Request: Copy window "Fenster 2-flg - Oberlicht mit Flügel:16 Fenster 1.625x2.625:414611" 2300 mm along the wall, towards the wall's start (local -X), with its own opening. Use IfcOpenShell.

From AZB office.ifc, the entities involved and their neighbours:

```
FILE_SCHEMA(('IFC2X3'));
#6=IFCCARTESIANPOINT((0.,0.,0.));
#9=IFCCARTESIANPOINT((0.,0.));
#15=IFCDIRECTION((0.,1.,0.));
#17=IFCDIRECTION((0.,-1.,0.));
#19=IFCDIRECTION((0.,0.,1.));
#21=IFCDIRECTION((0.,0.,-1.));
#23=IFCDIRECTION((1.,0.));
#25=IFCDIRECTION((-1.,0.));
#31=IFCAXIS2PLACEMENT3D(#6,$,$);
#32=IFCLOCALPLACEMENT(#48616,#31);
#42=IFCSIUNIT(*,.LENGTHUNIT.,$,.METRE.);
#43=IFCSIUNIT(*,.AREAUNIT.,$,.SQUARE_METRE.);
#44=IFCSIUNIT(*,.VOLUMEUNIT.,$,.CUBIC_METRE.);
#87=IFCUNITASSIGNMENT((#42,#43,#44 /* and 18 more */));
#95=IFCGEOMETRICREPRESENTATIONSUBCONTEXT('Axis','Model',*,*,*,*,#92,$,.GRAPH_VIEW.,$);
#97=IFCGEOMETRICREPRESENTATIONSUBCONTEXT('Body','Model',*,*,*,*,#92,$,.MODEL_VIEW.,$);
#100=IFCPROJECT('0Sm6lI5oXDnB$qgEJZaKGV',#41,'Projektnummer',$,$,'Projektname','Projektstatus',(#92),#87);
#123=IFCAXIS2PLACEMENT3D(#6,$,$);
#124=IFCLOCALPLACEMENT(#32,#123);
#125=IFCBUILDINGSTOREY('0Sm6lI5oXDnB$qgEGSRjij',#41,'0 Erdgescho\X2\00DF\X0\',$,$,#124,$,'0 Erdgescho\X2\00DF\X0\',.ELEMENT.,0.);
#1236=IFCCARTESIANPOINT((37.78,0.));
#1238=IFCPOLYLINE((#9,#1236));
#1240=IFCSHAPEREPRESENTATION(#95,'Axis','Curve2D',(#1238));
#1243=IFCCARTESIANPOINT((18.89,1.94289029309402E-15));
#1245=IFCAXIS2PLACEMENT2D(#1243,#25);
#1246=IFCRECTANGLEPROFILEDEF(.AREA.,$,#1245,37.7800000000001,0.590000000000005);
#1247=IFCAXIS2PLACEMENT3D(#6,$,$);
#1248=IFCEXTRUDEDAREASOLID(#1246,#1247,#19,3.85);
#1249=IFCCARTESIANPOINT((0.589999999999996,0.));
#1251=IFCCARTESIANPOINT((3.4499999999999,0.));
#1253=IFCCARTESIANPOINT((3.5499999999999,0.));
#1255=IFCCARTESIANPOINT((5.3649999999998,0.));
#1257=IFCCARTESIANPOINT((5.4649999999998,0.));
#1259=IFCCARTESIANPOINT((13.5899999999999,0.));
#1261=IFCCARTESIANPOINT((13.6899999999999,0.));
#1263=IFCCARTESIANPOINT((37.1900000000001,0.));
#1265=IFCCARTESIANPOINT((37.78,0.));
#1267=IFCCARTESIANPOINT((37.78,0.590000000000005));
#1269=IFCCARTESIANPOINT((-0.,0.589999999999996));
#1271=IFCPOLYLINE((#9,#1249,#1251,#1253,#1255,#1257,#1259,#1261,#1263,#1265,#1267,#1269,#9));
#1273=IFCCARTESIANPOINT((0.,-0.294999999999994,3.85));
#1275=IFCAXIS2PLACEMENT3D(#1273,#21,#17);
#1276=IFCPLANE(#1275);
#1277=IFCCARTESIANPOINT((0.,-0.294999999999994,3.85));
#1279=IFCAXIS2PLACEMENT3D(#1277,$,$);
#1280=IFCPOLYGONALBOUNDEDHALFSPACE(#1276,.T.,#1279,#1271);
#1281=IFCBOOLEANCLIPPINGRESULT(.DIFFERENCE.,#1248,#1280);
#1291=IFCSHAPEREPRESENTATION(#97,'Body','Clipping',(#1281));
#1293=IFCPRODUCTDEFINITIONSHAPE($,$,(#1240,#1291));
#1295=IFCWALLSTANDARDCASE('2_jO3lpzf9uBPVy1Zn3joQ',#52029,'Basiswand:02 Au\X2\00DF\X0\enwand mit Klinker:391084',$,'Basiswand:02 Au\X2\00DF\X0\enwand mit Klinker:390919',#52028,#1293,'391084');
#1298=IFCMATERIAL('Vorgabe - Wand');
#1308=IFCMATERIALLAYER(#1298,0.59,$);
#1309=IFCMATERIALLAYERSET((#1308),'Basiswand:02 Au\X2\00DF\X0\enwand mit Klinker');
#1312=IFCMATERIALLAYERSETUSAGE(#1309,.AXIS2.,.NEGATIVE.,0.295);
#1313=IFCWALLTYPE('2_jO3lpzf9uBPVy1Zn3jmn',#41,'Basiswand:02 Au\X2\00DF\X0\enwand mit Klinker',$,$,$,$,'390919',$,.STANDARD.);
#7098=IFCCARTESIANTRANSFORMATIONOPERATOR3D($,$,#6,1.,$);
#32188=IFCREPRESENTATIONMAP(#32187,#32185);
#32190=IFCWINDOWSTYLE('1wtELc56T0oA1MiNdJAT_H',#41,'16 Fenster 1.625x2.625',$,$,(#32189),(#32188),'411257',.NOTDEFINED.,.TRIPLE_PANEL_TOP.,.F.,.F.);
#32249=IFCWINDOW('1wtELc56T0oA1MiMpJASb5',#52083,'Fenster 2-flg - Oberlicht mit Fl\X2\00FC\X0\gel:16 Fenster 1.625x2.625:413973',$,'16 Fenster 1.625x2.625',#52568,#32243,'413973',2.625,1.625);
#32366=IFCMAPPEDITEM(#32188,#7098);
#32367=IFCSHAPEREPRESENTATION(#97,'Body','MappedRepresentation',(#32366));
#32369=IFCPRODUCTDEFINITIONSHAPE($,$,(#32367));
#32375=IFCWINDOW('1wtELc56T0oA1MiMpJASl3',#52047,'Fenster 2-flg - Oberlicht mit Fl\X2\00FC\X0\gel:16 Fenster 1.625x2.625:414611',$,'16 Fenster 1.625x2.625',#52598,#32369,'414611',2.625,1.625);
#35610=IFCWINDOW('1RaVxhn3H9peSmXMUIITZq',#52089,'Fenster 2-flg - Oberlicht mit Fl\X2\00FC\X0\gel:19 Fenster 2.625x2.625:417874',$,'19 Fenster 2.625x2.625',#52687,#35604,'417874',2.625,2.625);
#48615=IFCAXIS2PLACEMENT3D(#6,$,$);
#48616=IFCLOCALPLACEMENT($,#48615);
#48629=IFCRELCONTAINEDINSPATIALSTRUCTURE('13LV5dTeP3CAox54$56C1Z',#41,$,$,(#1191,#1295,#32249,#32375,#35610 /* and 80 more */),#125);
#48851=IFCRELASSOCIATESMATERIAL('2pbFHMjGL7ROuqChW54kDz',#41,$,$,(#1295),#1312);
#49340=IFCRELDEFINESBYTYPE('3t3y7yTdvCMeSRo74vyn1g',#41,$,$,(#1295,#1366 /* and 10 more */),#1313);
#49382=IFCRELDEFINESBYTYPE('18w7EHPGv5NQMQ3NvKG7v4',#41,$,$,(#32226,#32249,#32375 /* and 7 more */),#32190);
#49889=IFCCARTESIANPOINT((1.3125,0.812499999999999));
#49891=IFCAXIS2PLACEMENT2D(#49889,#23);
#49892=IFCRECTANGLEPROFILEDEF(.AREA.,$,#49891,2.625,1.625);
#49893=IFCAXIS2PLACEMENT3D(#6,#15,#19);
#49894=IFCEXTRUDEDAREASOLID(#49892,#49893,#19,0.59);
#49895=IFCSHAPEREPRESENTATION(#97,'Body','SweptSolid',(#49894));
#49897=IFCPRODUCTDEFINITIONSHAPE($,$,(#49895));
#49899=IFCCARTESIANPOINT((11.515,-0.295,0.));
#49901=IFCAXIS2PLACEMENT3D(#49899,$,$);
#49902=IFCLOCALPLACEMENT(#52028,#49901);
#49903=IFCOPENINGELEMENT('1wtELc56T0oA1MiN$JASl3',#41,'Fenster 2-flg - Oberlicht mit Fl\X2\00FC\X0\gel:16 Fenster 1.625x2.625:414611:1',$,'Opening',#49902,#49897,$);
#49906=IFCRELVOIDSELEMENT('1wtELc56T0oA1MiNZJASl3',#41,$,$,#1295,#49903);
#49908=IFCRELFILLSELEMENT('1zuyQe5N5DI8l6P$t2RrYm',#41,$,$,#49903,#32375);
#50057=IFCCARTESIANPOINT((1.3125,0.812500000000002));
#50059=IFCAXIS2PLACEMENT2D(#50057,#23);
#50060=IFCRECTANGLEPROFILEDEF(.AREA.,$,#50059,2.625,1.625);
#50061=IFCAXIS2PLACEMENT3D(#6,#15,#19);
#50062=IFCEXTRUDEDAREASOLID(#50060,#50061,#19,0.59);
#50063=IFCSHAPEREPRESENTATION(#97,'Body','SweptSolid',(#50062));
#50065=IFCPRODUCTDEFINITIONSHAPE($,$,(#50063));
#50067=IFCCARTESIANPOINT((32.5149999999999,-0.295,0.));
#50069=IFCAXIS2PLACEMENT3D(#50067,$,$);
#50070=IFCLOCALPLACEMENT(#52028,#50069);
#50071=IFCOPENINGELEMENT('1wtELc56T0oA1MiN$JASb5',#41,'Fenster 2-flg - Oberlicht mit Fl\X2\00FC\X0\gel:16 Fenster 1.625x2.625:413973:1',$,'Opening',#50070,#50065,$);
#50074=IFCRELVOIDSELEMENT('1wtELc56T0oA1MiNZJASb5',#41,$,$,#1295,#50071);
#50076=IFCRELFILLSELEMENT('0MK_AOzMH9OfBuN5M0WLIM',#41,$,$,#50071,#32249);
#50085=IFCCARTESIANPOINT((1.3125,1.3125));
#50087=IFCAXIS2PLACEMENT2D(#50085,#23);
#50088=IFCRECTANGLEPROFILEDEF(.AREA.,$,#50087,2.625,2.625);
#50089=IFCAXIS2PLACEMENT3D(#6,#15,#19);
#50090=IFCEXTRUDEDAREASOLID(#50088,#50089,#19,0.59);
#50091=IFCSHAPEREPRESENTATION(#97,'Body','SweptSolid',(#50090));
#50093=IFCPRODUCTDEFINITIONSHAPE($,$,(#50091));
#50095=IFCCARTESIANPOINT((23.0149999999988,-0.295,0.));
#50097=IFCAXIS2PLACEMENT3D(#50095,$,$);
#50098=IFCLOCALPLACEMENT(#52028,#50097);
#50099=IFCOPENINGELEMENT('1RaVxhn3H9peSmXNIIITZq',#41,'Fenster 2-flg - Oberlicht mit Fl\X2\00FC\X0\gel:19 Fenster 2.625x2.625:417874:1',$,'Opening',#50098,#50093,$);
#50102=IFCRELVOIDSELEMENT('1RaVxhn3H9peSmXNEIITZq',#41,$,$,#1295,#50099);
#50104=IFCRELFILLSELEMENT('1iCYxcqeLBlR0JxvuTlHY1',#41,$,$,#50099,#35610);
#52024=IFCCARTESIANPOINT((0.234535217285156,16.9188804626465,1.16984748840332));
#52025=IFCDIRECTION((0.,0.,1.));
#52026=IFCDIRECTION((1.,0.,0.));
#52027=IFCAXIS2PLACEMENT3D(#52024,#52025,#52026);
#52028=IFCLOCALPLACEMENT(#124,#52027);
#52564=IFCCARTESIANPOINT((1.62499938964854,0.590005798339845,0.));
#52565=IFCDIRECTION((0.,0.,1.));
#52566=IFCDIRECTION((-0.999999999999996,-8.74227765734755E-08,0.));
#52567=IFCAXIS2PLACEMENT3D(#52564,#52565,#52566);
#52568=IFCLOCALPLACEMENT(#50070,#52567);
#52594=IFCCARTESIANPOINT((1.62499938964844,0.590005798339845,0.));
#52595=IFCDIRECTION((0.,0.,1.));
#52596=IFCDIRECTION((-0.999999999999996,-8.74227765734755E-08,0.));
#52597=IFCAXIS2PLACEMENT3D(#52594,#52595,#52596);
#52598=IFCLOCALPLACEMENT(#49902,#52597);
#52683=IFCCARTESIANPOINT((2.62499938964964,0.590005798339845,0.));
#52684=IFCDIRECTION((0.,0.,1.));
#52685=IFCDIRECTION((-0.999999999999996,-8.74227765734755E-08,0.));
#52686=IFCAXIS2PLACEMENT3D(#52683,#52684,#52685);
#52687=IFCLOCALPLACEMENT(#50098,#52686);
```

```python
import ifcopenshell
import ifcopenshell.api.feature
import ifcopenshell.api.geometry
import ifcopenshell.api.root
import ifcopenshell.geom
import ifcopenshell.util.element
import ifcopenshell.util.placement
import ifcopenshell.util.shape

model = ifcopenshell.open("AZB office.ifc")
settings = ifcopenshell.geom.settings()


def volume(element):
    """Net volume in cubic metres, openings subtracted."""
    shape = ifcopenshell.geom.create_shape(settings, element)
    return ifcopenshell.util.shape.get_volume(shape.geometry)


def reuse_history(source, copy):
    """copy_class also copies each property set's owner history, people and application; keep the originals."""
    for rel in copy.IsDefinedBy:
        if rel.is_a("IfcRelDefinesByProperties") and (history := rel.RelatingPropertyDefinition.OwnerHistory):
            rel.RelatingPropertyDefinition.OwnerHistory = source.OwnerHistory
            ifcopenshell.util.element.remove_deep2(model, history)


window = model.by_id(32375)
opening = window.FillsVoids[0].RelatingOpeningElement
wall = opening.VoidsElements[0].RelatingBuildingElement
before = volume(wall)
shift = ifcopenshell.util.placement.get_local_placement(wall.ObjectPlacement)[:3, 0] * -2.3

# copy_class copies the void relationship, type, container and properties, but no geometry.
new_opening = ifcopenshell.api.root.copy_class(model, product=opening)
new_opening.Representation = ifcopenshell.util.element.copy_deep(
    model, opening.Representation, exclude=["IfcGeometricRepresentationContext", "IfcRepresentationMap"]
)
new_opening.Name = "Fenster 2-flg - Oberlicht mit Flügel:16 Fenster 1.625x2.625"
new_window = ifcopenshell.api.root.copy_class(model, product=window)
new_window.Representation = ifcopenshell.util.element.copy_deep(
    model, window.Representation, exclude=["IfcGeometricRepresentationContext", "IfcRepresentationMap"]
)
new_window.Name = "Fenster 2-flg - Oberlicht mit Flügel:16 Fenster 1.625x2.625"
new_window.Tag = None
reuse_history(window, new_window)
fills = ifcopenshell.api.feature.add_filling(model, opening=new_opening, element=new_window)
fills.OwnerHistory = new_window.OwnerHistory  # required in IFC2X3

for old, new in ((opening, new_opening), (window, new_window)):
    matrix = ifcopenshell.util.placement.get_local_placement(old.ObjectPlacement)
    matrix[:3, 3] += shift
    ifcopenshell.api.geometry.edit_object_placement(model, product=new, matrix=matrix, is_si=False)

after = volume(wall)

print(f"wall volume {before:.3f} -> {after:.3f} m3")

model.write("AZB office_v2.ifc")
```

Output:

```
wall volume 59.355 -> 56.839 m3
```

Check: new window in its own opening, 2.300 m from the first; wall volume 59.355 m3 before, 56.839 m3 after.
